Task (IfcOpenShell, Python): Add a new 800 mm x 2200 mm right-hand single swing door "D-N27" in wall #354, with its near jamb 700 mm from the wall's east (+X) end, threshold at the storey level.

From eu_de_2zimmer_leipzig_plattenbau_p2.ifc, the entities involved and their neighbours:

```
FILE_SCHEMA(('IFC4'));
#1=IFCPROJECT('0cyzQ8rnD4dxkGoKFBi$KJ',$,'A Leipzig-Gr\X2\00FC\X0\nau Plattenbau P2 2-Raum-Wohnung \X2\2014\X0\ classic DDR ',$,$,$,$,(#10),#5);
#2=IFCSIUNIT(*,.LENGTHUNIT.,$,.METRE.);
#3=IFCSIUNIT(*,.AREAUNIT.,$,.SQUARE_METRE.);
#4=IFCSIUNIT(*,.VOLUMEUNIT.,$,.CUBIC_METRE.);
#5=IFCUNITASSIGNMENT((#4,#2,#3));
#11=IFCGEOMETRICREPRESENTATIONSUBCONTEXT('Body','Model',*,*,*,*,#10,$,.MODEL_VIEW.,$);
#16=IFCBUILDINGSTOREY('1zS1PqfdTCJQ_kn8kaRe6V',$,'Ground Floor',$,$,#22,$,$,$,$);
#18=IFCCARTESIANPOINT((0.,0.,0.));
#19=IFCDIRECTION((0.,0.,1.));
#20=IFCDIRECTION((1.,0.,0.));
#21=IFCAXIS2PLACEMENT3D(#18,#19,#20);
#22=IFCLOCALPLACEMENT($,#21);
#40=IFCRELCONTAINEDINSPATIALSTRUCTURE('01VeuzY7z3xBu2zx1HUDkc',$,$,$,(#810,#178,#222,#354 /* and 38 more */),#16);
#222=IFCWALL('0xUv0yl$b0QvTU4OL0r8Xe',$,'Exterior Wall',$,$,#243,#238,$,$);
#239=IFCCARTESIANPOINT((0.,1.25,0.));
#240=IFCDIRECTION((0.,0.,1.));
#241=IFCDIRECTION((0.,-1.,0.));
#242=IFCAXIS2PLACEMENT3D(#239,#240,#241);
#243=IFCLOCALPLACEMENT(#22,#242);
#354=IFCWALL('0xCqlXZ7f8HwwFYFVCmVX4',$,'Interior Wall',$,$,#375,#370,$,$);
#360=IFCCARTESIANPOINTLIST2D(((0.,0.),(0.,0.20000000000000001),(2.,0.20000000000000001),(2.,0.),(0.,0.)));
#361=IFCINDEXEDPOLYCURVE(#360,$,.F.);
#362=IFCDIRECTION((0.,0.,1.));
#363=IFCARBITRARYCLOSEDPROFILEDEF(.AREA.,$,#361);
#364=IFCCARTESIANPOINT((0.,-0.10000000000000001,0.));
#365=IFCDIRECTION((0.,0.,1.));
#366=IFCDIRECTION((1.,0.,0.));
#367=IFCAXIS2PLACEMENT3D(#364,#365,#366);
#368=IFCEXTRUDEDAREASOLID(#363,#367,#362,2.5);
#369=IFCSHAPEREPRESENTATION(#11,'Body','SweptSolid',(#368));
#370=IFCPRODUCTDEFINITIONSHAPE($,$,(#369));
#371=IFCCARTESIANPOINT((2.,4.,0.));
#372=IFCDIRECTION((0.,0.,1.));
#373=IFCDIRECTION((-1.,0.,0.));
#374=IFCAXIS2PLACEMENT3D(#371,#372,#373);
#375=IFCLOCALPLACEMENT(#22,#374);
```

```python
import numpy as np
import ifcopenshell
import ifcopenshell.api.feature
import ifcopenshell.api.geometry
import ifcopenshell.api.root
import ifcopenshell.api.spatial
import ifcopenshell.geom
import ifcopenshell.util.element
import ifcopenshell.util.placement
import ifcopenshell.util.representation
import ifcopenshell.util.shape
import ifcopenshell.util.unit

model = ifcopenshell.open("eu_de_2zimmer_leipzig_plattenbau_p2.ifc")
unit_scale = ifcopenshell.util.unit.calculate_unit_scale(model)
settings = ifcopenshell.geom.settings()


def volume(element):
    """Net volume in cubic metres, openings subtracted."""
    shape = ifcopenshell.geom.create_shape(settings, element)
    return ifcopenshell.util.shape.get_volume(shape.geometry)


wall = model.by_id(354)
storey = ifcopenshell.util.element.get_container(wall, ifc_class="IfcBuildingStorey")
context = ifcopenshell.util.representation.get_context(model, "Model", "Body", "MODEL_VIEW")
before = volume(wall)

width, height, from_end, sill = 0.8, 2.2, 0.7, 0.0  # metres

# The wall runs along its own X axis, and the end named is its -X end.
wall_shape = ifcopenshell.geom.create_shape(settings, wall)
x, y, z = ifcopenshell.util.shape.get_vertices(wall_shape.geometry).T
start = x.min() + from_end
face, thickness = float(y.min()), float(y.max() - y.min())
wall_matrix = ifcopenshell.util.placement.get_local_placement(wall.ObjectPlacement)
level = ifcopenshell.util.placement.get_local_placement(storey.ObjectPlacement)[2, 3]


def in_wall(x, y):
    """Placement at x, y metres in the wall's axes, at sill height."""
    matrix = wall_matrix.copy()
    matrix[:, 3] = wall_matrix @ np.array([x / unit_scale, y / unit_scale, 0.0, 1.0])
    matrix[2, 3] = level + sill / unit_scale
    return matrix


# Opening: a box that overshoots both wall faces by 50 mm.
opening = ifcopenshell.api.root.create_entity(model, ifc_class="IfcOpeningElement", predefined_type="OPENING")
box = ifcopenshell.api.geometry.add_wall_representation(
    model, context=context, length=width, height=height, thickness=thickness + 0.1
)
ifcopenshell.api.geometry.assign_representation(model, product=opening, representation=box)
ifcopenshell.api.geometry.edit_object_placement(model, product=opening, matrix=in_wall(start, face - 0.05), is_si=False)
ifcopenshell.api.feature.add_feature(model, feature=opening, element=wall)

door = ifcopenshell.api.root.create_entity(model, ifc_class="IfcDoor", name="D-N27", predefined_type="DOOR")
door.OverallWidth, door.OverallHeight = width / unit_scale, height / unit_scale
door.OperationType = "SINGLE_SWING_RIGHT"
body = ifcopenshell.api.geometry.add_door_representation(
    model,
    context=context,
    overall_width=door.OverallWidth,
    overall_height=door.OverallHeight,
    operation_type="SINGLE_SWING_RIGHT",
    lining_properties={"LiningDepth": thickness / unit_scale, "ThresholdDepth": thickness / unit_scale},
)
ifcopenshell.api.geometry.assign_representation(model, product=door, representation=body)
ifcopenshell.api.spatial.assign_container(model, products=[door], relating_structure=storey)
ifcopenshell.api.feature.add_filling(model, opening=opening, element=door)

# The lining spans the wall, so the door starts at the wall face.
ifcopenshell.api.geometry.edit_object_placement(model, product=door, matrix=in_wall(start, face), is_si=False)

after = volume(wall)

print(f"wall volume {before:.3f} -> {after:.3f} m3")

model.write("eu_de_2zimmer_leipzig_plattenbau_p2-out.ifc")
```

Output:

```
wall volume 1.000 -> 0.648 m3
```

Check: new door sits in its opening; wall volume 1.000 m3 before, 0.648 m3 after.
